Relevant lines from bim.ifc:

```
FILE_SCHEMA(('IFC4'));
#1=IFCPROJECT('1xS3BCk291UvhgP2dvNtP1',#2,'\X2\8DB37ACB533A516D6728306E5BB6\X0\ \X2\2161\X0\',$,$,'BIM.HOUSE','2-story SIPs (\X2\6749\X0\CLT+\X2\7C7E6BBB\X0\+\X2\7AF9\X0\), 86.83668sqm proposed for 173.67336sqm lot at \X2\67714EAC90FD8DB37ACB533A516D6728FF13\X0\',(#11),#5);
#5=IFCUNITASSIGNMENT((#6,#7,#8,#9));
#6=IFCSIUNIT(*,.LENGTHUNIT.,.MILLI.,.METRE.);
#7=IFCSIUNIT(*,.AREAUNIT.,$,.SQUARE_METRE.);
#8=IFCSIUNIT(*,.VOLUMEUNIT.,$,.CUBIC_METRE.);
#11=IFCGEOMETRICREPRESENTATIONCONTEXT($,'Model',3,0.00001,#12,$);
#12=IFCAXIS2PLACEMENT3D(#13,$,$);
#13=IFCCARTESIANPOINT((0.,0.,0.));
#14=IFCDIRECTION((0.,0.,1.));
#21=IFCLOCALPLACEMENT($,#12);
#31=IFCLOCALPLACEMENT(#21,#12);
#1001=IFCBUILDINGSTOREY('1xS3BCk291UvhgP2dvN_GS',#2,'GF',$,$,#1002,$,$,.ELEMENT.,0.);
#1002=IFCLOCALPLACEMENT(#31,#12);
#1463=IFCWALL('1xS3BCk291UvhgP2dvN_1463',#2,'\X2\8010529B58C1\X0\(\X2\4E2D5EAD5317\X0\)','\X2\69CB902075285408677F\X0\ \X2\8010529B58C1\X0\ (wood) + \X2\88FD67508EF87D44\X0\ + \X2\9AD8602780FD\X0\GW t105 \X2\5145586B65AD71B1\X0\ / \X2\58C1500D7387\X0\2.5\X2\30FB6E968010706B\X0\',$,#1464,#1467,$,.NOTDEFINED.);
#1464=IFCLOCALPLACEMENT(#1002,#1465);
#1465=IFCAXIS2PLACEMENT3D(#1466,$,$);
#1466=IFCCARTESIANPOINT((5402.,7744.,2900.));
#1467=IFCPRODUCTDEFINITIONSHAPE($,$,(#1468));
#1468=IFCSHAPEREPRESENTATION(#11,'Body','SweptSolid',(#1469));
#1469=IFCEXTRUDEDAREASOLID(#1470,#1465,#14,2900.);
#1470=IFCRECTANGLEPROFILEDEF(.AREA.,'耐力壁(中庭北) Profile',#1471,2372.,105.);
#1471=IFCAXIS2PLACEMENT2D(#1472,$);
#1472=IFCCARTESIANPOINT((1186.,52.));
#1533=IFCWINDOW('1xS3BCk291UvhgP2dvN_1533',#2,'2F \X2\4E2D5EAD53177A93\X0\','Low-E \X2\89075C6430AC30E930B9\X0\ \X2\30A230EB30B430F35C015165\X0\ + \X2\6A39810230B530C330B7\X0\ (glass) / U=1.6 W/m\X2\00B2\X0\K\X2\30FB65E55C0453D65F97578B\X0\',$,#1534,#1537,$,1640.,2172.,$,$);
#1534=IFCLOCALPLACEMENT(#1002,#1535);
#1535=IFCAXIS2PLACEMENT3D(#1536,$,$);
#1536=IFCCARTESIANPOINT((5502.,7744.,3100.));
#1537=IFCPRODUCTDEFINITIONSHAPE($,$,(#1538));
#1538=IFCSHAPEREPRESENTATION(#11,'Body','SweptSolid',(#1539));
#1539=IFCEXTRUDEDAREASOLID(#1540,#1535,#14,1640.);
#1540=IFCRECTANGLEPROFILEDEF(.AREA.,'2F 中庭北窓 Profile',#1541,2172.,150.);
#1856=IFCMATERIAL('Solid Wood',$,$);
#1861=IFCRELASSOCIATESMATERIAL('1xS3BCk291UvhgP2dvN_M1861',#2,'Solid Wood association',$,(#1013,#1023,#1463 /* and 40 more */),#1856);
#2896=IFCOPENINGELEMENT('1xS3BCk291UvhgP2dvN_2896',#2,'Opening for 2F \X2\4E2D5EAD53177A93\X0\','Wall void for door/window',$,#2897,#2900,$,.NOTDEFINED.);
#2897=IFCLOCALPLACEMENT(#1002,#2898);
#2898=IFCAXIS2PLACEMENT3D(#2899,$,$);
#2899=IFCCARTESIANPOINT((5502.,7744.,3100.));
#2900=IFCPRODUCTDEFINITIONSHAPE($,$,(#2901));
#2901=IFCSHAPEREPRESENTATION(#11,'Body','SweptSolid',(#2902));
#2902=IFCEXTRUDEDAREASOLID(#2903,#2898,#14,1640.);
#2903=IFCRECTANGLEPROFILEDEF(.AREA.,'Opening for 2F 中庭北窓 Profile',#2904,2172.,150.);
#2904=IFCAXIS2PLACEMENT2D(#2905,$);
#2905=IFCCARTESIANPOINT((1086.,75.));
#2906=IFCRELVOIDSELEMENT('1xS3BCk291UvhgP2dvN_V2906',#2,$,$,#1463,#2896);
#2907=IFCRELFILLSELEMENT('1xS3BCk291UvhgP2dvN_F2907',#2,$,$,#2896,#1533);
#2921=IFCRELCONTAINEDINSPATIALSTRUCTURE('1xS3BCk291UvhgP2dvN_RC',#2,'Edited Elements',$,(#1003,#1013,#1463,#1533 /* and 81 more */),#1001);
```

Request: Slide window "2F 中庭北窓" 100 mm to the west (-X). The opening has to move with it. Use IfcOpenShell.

```python
import ifcopenshell
import ifcopenshell.api.geometry
import ifcopenshell.util.placement
import ifcopenshell.util.unit

model = ifcopenshell.open("bim.ifc")
unit_scale = ifcopenshell.util.unit.calculate_unit_scale(model)

window = model.by_guid("1xS3BCk291UvhgP2dvN_1533")
opening = window.FillsVoids[0].RelatingOpeningElement
wall = opening.VoidsElements[0].RelatingBuildingElement

wall_matrix = ifcopenshell.util.placement.get_local_placement(wall.ObjectPlacement)
shift = wall_matrix[:3, 0] * -0.1 / unit_scale
before = ifcopenshell.util.placement.get_local_placement(window.ObjectPlacement)[:3, 3].copy()

# The window is not placed relative to its opening, so move both.
for product in (opening, window):
    matrix = ifcopenshell.util.placement.get_local_placement(product.ObjectPlacement)
    matrix[:3, 3] += shift
    ifcopenshell.api.geometry.edit_object_placement(model, product=product, matrix=matrix, is_si=False)

after = ifcopenshell.util.placement.get_local_placement(window.ObjectPlacement)[:3, 3]
print("window moved by", (after - before).round(3) + 0.0)

model.write("bim_v2.ifc")
```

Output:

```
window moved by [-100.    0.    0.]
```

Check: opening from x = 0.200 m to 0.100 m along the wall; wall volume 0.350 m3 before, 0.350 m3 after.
